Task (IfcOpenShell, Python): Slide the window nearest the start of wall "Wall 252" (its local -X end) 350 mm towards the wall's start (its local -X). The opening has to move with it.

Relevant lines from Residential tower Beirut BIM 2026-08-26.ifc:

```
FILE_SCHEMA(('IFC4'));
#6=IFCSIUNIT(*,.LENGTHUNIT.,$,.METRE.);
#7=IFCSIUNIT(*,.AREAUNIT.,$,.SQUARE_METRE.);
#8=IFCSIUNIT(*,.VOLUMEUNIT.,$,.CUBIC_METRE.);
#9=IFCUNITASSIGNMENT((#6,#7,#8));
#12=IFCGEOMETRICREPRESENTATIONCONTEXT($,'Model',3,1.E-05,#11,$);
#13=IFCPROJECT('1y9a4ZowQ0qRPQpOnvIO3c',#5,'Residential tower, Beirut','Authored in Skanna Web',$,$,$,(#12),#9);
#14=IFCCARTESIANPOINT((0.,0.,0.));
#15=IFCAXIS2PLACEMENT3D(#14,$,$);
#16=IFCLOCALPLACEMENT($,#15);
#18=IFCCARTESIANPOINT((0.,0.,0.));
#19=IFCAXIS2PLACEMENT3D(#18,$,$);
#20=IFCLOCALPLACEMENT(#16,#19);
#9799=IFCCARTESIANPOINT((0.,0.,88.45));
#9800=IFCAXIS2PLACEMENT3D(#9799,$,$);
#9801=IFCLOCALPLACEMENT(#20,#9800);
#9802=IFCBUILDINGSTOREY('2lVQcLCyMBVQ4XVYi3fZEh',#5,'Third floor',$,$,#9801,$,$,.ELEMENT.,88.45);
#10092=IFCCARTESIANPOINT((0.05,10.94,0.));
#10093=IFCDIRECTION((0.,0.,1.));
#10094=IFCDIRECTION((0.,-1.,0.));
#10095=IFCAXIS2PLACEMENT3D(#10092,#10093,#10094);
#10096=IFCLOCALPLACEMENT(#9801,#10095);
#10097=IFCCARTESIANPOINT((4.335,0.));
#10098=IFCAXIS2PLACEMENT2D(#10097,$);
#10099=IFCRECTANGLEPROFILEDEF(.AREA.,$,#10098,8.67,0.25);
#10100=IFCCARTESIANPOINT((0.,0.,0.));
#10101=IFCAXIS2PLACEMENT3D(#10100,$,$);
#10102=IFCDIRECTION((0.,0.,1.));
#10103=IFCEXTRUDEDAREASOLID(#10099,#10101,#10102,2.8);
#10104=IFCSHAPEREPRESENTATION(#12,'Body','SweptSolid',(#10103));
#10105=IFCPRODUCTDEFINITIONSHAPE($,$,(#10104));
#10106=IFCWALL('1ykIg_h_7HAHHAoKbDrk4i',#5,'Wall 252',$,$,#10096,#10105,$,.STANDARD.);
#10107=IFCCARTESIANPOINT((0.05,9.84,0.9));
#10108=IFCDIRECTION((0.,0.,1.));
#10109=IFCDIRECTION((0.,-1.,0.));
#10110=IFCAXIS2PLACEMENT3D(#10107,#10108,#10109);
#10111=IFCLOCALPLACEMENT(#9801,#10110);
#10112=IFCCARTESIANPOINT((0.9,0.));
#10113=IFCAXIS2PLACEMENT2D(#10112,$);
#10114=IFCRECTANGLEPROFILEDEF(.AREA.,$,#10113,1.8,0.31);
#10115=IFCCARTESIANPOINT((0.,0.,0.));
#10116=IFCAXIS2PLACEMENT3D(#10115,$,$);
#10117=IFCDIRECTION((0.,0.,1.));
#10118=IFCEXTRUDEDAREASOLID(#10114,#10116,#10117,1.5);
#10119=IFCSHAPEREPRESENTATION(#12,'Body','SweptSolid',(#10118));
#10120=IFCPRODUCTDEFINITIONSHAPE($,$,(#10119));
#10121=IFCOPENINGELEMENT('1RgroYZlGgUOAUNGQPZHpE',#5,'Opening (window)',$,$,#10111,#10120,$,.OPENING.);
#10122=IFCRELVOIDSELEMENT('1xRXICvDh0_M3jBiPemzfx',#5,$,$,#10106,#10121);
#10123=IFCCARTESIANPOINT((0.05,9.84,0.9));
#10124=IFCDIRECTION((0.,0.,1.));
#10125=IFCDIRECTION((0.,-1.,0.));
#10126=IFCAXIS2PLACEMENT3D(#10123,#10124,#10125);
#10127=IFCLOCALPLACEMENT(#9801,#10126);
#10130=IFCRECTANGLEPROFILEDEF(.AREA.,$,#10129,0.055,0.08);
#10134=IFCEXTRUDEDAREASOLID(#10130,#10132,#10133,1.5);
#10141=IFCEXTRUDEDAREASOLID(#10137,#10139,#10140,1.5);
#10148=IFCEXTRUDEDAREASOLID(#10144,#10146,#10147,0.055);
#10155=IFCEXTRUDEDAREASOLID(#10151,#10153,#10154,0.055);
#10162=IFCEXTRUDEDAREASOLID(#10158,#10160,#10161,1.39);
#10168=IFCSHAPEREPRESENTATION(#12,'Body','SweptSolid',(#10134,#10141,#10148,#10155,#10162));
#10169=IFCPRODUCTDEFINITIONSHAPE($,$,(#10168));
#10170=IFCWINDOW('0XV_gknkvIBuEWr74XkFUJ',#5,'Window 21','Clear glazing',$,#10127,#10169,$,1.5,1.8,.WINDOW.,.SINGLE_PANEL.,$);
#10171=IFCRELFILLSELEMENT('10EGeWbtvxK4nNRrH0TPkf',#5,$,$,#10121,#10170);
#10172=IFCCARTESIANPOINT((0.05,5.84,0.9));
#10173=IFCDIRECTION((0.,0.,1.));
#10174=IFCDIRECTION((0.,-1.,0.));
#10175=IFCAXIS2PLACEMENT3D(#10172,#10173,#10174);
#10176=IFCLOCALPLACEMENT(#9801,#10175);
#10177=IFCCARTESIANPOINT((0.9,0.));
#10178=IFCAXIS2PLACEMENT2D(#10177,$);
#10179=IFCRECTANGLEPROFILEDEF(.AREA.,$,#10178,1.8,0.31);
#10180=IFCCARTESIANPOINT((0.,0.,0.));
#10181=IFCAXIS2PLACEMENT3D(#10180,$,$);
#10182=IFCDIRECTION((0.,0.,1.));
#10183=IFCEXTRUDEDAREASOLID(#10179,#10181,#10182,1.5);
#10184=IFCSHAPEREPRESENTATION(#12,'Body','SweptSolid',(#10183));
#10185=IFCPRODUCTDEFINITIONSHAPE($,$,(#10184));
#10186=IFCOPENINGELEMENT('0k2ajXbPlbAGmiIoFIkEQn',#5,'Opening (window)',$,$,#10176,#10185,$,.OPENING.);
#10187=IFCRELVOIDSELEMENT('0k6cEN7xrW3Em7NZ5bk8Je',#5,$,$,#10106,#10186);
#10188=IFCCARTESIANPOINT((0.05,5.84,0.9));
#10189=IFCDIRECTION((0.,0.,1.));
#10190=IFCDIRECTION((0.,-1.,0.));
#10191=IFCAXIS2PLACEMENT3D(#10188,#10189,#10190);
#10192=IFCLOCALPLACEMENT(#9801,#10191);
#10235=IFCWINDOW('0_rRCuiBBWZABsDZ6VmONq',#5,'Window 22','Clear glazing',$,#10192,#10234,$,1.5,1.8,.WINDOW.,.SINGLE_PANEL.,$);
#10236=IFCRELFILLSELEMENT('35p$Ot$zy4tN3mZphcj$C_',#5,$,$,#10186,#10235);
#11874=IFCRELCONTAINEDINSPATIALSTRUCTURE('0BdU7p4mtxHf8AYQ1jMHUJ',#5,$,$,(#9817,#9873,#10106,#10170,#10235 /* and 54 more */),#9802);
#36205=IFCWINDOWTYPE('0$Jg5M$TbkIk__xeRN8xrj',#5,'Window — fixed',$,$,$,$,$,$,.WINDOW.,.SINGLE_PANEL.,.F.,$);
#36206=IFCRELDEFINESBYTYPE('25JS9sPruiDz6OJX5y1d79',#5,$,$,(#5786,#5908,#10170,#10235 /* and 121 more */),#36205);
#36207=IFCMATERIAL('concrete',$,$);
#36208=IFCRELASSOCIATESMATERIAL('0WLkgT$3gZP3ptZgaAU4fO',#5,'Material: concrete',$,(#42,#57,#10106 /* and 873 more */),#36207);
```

```python
import ifcopenshell
import ifcopenshell.api.geometry
import ifcopenshell.util.placement
import ifcopenshell.util.unit

model = ifcopenshell.open("Residential tower Beirut BIM 2026-08-26.ifc")
unit_scale = ifcopenshell.util.unit.calculate_unit_scale(model)

window = model.by_guid("0XV_gknkvIBuEWr74XkFUJ")
opening = window.FillsVoids[0].RelatingOpeningElement
wall = opening.VoidsElements[0].RelatingBuildingElement

wall_matrix = ifcopenshell.util.placement.get_local_placement(wall.ObjectPlacement)
shift = wall_matrix[:3, 0] * -0.35 / unit_scale
before = ifcopenshell.util.placement.get_local_placement(window.ObjectPlacement)[:3, 3].copy()

# The window is not placed relative to its opening, so move both.
for product in (opening, window):
    matrix = ifcopenshell.util.placement.get_local_placement(product.ObjectPlacement)
    matrix[:3, 3] += shift
    ifcopenshell.api.geometry.edit_object_placement(model, product=product, matrix=matrix, is_si=False)

after = ifcopenshell.util.placement.get_local_placement(window.ObjectPlacement)[:3, 3]
print("window moved by", (after - before).round(3) + 0.0)

model.write("Residential tower Beirut BIM 2026-08-26_updated.ifc")
```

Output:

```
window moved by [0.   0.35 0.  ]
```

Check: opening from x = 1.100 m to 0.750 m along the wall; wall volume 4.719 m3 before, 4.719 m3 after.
